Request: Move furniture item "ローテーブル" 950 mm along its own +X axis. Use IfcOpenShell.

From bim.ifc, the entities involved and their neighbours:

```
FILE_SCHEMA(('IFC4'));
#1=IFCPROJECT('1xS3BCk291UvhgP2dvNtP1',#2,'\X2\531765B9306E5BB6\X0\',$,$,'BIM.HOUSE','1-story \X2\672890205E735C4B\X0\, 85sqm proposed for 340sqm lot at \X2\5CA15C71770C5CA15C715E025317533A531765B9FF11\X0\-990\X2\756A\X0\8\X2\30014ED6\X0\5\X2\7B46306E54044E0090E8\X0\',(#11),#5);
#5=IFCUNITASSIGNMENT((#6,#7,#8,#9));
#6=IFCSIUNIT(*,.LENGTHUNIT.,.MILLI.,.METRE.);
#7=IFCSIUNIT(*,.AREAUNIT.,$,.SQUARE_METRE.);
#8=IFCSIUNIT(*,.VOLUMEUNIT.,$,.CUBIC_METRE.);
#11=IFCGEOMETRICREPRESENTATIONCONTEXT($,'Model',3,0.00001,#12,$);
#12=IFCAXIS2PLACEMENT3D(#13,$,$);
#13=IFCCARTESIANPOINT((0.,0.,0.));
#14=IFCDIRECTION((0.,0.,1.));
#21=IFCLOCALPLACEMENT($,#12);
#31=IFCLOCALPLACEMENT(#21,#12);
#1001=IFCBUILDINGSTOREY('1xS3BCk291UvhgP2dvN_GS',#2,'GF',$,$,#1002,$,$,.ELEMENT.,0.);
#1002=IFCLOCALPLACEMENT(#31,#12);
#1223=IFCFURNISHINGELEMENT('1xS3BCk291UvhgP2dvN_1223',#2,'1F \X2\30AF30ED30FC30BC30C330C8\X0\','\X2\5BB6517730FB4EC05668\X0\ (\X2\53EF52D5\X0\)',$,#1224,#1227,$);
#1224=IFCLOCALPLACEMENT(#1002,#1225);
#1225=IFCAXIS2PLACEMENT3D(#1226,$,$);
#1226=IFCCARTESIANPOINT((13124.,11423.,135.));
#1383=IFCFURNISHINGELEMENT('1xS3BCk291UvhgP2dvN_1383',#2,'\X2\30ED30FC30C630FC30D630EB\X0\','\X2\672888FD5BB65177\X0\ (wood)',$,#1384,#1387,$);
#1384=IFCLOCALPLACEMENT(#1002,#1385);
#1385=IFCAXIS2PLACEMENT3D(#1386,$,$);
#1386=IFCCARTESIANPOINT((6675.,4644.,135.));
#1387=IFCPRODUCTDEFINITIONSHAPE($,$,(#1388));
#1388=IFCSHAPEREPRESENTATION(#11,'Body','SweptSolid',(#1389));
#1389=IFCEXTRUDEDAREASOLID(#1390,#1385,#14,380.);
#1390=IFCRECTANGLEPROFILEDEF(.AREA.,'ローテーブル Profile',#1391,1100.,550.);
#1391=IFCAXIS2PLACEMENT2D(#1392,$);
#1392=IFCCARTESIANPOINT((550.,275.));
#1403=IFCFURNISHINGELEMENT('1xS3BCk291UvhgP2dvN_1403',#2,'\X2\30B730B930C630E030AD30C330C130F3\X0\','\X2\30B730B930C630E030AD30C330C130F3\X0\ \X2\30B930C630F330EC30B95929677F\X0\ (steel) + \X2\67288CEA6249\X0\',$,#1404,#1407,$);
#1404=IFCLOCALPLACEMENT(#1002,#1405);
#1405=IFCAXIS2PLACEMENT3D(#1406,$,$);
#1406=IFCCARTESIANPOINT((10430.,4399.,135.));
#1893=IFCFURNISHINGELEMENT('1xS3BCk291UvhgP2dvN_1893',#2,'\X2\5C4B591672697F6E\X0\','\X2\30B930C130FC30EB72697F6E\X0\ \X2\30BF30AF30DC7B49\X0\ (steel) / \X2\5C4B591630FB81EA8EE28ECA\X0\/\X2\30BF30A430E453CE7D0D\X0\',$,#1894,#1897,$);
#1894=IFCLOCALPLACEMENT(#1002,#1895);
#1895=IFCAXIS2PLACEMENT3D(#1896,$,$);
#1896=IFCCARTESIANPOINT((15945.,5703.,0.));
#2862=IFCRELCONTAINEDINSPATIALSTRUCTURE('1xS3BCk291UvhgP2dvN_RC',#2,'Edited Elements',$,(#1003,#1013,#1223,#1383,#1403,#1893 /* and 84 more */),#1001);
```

```python
import ifcopenshell
import ifcopenshell.api.geometry
import ifcopenshell.util.placement
import ifcopenshell.util.unit

model = ifcopenshell.open("bim.ifc")
unit_scale = ifcopenshell.util.unit.calculate_unit_scale(model)

item = model.by_id(1383)
matrix = ifcopenshell.util.placement.get_local_placement(item.ObjectPlacement)
matrix[:3, 3] += matrix[:3, 0] * 0.95 / unit_scale
ifcopenshell.api.geometry.edit_object_placement(model, product=item, matrix=matrix, is_si=False)

print(ifcopenshell.util.placement.get_local_placement(item.ObjectPlacement).round(3) + 0.0)

model.write("bim-out.ifc")
```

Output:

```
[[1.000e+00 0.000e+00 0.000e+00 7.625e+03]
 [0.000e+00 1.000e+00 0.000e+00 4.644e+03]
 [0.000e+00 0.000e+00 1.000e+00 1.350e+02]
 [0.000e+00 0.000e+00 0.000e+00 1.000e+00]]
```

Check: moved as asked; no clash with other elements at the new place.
